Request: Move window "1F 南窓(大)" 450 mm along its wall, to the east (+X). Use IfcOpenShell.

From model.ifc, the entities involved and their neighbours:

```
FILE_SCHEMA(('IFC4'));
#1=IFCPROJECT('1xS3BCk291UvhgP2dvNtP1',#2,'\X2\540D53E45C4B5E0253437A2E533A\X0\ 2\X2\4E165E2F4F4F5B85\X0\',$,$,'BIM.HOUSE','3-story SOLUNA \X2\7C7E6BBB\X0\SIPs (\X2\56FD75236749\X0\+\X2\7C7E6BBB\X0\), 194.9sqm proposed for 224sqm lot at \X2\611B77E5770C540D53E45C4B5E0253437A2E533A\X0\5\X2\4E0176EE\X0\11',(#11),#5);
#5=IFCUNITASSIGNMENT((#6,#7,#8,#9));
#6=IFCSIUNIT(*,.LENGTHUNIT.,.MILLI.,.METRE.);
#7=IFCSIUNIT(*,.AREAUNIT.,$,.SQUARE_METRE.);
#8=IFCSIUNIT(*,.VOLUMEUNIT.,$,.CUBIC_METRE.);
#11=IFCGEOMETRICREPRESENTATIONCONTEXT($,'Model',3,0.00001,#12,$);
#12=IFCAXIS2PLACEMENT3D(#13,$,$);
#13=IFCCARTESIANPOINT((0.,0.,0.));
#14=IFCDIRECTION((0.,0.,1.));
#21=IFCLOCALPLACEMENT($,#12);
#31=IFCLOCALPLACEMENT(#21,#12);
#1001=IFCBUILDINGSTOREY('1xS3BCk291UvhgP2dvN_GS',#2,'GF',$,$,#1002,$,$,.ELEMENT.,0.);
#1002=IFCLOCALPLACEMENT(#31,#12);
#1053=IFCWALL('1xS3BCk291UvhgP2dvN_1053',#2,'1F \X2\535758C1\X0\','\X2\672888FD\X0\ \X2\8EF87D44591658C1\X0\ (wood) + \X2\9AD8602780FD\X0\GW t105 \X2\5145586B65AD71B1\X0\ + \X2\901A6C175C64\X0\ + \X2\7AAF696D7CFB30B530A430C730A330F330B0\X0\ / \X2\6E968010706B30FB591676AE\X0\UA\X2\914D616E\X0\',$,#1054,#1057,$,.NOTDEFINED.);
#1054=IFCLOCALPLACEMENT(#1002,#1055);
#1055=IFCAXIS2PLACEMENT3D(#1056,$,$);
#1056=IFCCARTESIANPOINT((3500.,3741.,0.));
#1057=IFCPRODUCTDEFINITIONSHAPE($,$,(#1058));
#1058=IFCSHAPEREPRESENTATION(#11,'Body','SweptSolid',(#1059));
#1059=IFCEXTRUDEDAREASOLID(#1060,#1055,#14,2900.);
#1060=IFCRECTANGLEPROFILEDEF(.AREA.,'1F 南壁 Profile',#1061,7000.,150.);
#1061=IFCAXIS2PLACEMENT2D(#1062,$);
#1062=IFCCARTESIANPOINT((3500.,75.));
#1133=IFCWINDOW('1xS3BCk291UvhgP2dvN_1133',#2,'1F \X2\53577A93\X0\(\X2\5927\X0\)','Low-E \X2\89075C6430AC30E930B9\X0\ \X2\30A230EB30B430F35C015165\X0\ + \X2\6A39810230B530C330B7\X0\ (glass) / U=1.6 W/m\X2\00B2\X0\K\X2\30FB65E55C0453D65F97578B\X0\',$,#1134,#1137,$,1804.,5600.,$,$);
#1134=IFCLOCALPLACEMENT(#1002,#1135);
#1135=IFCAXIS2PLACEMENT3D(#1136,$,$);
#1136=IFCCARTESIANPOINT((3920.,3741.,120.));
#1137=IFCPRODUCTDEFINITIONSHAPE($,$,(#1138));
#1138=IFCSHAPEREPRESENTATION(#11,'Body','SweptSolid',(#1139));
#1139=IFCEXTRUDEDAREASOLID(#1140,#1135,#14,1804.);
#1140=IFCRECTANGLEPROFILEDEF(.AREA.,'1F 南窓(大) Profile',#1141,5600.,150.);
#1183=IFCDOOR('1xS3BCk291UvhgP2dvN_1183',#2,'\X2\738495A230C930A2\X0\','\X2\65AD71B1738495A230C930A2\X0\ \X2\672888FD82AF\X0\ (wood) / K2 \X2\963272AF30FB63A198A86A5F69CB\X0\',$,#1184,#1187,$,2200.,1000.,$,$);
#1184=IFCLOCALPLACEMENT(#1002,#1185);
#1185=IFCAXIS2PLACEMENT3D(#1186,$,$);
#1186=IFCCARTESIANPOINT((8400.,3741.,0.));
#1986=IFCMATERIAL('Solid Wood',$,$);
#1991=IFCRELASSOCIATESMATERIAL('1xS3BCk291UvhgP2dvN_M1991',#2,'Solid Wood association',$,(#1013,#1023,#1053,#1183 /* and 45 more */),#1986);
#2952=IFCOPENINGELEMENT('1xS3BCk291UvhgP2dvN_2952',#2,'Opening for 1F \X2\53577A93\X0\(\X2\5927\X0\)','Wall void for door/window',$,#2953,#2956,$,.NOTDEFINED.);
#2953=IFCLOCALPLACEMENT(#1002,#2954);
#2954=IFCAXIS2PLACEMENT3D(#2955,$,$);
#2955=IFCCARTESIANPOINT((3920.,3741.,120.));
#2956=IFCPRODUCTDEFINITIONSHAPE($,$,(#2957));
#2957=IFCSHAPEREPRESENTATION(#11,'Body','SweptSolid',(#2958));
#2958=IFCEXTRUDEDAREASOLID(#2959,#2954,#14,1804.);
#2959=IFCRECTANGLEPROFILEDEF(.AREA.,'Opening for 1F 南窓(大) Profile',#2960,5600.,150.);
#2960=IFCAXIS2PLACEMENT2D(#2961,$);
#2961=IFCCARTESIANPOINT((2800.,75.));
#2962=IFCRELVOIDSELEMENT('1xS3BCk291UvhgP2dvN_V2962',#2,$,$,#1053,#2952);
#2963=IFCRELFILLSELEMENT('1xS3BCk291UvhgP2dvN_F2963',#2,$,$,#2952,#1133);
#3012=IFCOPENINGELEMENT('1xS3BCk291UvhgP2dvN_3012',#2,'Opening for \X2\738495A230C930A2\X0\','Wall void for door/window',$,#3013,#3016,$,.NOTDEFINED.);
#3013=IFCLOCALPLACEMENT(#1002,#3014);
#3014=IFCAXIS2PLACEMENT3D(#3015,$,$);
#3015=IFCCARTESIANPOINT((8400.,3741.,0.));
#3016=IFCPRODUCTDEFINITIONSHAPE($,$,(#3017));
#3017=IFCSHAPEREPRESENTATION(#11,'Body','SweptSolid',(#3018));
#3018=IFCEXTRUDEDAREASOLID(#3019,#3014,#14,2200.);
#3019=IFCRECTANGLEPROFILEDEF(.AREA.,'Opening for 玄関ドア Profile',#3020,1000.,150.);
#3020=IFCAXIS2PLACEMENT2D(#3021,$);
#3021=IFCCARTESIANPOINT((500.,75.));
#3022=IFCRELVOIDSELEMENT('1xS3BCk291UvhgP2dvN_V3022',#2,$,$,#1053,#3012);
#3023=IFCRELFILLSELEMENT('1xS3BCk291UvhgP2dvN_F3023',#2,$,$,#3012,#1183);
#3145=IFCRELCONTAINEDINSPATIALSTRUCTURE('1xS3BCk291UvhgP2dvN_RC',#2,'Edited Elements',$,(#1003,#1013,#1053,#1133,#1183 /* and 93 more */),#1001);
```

```python
import ifcopenshell
import ifcopenshell.api.geometry
import ifcopenshell.util.placement
import ifcopenshell.util.unit

model = ifcopenshell.open("model.ifc")
unit_scale = ifcopenshell.util.unit.calculate_unit_scale(model)

window = model.by_id(1133)
opening = window.FillsVoids[0].RelatingOpeningElement
wall = opening.VoidsElements[0].RelatingBuildingElement

wall_matrix = ifcopenshell.util.placement.get_local_placement(wall.ObjectPlacement)
shift = wall_matrix[:3, 0] * 0.45 / unit_scale
before = ifcopenshell.util.placement.get_local_placement(window.ObjectPlacement)[:3, 3].copy()

# The window is not placed relative to its opening, so move both.
for product in (opening, window):
    matrix = ifcopenshell.util.placement.get_local_placement(product.ObjectPlacement)
    matrix[:3, 3] += shift
    ifcopenshell.api.geometry.edit_object_placement(model, product=product, matrix=matrix, is_si=False)

after = ifcopenshell.util.placement.get_local_placement(window.ObjectPlacement)[:3, 3]
print("window moved by", (after - before).round(3) + 0.0)

model.write("model_rev.ifc")
```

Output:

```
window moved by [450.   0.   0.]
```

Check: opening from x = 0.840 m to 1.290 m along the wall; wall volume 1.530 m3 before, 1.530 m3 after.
